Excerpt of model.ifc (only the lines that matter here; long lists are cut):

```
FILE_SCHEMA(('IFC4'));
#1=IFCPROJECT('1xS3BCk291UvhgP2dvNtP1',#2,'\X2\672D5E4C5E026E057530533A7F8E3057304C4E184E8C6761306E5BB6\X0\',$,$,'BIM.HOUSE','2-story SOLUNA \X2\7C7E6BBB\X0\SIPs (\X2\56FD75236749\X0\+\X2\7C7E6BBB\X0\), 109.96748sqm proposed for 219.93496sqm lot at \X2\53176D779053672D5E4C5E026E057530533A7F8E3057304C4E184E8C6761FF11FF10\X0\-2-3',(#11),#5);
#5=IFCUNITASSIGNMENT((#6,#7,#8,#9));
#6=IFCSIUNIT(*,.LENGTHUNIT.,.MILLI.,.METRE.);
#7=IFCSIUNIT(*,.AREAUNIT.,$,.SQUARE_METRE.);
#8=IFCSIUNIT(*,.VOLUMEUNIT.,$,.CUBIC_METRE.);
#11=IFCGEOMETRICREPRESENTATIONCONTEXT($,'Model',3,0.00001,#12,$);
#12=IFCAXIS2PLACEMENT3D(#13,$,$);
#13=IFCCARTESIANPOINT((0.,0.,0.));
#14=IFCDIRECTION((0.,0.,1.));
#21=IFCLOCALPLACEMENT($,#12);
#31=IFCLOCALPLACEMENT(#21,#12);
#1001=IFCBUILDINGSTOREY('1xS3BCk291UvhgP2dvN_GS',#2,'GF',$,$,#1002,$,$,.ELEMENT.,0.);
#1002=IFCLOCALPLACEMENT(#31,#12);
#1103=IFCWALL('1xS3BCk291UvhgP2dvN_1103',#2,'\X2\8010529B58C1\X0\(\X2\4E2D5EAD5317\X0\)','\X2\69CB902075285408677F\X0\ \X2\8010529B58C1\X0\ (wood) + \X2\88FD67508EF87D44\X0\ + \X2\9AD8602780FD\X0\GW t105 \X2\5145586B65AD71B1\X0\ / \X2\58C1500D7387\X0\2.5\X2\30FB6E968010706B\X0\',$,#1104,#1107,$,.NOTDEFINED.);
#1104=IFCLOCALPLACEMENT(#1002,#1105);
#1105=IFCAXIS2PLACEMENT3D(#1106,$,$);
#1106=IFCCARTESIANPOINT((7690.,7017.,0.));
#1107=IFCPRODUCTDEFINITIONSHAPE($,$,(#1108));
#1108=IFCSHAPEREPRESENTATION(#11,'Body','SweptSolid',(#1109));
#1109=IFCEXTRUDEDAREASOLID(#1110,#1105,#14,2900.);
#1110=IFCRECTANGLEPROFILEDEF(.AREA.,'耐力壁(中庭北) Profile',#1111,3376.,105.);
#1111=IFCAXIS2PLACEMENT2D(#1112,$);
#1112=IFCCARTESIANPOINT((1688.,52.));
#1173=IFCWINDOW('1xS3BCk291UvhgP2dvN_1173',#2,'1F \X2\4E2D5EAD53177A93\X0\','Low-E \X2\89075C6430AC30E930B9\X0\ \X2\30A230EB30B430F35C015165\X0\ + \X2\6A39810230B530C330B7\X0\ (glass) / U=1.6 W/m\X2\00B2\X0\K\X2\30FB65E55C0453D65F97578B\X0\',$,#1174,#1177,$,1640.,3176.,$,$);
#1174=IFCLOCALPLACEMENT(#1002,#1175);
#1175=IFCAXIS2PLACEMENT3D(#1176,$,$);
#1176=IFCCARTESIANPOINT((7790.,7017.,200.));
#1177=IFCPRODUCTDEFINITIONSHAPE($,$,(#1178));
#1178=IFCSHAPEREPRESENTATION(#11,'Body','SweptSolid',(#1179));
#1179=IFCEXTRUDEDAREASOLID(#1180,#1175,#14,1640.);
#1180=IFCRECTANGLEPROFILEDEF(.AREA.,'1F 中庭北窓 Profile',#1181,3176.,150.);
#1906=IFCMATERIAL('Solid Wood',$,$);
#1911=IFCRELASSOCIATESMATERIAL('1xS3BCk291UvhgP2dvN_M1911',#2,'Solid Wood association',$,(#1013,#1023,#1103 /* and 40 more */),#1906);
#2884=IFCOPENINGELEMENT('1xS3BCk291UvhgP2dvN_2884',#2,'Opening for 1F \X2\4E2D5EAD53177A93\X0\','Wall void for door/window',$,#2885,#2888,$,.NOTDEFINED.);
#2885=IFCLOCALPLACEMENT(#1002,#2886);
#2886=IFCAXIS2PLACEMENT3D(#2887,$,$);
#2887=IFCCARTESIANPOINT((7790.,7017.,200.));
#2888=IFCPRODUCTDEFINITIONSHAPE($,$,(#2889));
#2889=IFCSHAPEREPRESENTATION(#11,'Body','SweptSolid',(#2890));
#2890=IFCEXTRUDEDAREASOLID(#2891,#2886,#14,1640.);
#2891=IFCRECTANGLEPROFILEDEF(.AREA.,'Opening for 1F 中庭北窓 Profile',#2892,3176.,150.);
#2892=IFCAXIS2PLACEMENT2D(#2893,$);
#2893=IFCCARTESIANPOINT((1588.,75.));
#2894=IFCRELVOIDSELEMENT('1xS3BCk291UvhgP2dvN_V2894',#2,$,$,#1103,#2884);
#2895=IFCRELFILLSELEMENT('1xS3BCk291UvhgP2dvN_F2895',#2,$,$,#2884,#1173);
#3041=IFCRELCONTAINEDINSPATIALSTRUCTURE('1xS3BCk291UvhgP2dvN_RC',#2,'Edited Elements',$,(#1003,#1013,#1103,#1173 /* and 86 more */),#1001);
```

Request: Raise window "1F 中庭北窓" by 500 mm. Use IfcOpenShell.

```python
import numpy as np
import ifcopenshell
import ifcopenshell.api.geometry
import ifcopenshell.util.placement
import ifcopenshell.util.unit

model = ifcopenshell.open("model.ifc")
unit_scale = ifcopenshell.util.unit.calculate_unit_scale(model)

window = model.by_id(1173)
opening = window.FillsVoids[0].RelatingOpeningElement
dz = 500.0

shift = np.array([0.0, 0.0, dz])
# The window is not placed relative to its opening, so move both.
for product in (opening, window):
    matrix = ifcopenshell.util.placement.get_local_placement(product.ObjectPlacement)
    matrix[:3, 3] += shift
    ifcopenshell.api.geometry.edit_object_placement(model, product=product, matrix=matrix, is_si=False)

print(f"moved by {dz * unit_scale:+.3f} m")

model.write("model_edited.ifc")
```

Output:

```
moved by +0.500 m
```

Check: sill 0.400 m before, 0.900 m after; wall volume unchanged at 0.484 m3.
